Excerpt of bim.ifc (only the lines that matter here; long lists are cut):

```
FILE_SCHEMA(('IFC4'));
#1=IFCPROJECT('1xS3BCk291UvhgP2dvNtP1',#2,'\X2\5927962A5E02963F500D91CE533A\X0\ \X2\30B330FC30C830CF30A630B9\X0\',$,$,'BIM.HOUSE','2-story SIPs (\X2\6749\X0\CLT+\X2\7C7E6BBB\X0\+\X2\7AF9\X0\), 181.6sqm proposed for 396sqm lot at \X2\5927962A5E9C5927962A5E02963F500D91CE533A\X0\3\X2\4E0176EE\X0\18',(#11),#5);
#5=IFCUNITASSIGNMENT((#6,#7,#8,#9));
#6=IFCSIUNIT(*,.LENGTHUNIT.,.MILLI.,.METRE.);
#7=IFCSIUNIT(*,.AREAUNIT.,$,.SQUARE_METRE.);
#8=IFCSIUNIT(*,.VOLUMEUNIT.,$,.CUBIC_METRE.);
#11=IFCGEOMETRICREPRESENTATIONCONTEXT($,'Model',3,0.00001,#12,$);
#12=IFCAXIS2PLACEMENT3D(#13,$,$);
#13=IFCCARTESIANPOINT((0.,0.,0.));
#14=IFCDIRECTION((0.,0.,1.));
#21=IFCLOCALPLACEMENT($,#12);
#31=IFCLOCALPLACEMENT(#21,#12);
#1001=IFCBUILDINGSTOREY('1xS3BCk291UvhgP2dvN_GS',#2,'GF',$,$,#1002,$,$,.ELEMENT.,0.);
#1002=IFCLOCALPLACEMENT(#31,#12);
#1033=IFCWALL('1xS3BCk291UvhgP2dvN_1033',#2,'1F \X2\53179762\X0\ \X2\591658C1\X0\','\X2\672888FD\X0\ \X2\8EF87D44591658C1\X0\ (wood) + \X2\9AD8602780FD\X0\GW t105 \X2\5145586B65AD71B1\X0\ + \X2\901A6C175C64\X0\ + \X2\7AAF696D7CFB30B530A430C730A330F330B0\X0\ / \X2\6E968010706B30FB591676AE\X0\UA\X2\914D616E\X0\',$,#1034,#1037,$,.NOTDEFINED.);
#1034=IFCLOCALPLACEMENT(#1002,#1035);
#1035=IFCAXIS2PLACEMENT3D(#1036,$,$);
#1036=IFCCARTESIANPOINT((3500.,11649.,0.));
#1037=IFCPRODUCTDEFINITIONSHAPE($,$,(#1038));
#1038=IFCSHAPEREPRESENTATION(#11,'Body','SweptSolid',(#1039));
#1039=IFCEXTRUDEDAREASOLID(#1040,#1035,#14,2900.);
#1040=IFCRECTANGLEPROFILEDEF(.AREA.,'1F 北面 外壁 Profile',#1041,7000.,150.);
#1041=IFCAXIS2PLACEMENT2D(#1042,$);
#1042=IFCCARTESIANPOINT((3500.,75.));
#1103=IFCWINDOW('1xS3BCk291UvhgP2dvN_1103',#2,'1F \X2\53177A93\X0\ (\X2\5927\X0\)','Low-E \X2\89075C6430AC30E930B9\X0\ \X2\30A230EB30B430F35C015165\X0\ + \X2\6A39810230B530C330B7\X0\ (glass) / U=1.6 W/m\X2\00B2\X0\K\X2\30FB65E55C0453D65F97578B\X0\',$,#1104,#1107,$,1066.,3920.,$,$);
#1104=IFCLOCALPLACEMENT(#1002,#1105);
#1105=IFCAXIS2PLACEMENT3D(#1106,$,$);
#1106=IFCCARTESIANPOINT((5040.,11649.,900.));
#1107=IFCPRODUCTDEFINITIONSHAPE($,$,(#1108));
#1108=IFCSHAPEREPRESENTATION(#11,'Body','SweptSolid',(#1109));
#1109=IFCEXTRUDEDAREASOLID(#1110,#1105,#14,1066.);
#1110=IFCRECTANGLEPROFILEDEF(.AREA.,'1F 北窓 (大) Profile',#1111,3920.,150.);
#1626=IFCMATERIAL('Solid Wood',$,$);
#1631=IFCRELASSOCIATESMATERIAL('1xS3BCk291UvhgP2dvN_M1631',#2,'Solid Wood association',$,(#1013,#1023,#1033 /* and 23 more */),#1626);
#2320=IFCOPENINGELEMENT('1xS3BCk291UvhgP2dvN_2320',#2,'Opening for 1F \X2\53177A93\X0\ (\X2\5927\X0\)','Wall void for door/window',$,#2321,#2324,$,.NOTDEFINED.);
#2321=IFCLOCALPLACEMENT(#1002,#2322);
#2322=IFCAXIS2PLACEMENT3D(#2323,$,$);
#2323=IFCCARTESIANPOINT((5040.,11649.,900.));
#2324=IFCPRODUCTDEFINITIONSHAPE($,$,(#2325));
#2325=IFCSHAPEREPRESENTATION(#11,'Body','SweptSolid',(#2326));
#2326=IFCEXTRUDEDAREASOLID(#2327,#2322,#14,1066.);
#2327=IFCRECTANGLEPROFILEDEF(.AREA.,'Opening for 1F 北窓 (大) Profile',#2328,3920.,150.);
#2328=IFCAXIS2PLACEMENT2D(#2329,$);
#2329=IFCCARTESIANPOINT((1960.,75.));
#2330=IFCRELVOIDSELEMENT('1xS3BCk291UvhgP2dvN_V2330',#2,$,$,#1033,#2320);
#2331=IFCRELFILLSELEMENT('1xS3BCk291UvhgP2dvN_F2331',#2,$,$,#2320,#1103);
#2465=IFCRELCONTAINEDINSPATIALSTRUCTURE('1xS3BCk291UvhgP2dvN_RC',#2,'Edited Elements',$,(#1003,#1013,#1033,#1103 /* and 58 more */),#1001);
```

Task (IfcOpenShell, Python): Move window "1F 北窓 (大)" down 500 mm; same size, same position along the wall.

```python
import numpy as np
import ifcopenshell
import ifcopenshell.api.geometry
import ifcopenshell.util.placement
import ifcopenshell.util.unit

model = ifcopenshell.open("bim.ifc")
unit_scale = ifcopenshell.util.unit.calculate_unit_scale(model)

window = model.by_guid("1xS3BCk291UvhgP2dvN_1103")
opening = window.FillsVoids[0].RelatingOpeningElement
dz = -500.0

shift = np.array([0.0, 0.0, dz])
# The window is not placed relative to its opening, so move both.
for product in (opening, window):
    matrix = ifcopenshell.util.placement.get_local_placement(product.ObjectPlacement)
    matrix[:3, 3] += shift
    ifcopenshell.api.geometry.edit_object_placement(model, product=product, matrix=matrix, is_si=False)

print(f"moved by {dz * unit_scale:+.3f} m")

model.write("bim_updated.ifc")
```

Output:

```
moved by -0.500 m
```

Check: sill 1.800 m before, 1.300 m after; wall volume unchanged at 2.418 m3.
